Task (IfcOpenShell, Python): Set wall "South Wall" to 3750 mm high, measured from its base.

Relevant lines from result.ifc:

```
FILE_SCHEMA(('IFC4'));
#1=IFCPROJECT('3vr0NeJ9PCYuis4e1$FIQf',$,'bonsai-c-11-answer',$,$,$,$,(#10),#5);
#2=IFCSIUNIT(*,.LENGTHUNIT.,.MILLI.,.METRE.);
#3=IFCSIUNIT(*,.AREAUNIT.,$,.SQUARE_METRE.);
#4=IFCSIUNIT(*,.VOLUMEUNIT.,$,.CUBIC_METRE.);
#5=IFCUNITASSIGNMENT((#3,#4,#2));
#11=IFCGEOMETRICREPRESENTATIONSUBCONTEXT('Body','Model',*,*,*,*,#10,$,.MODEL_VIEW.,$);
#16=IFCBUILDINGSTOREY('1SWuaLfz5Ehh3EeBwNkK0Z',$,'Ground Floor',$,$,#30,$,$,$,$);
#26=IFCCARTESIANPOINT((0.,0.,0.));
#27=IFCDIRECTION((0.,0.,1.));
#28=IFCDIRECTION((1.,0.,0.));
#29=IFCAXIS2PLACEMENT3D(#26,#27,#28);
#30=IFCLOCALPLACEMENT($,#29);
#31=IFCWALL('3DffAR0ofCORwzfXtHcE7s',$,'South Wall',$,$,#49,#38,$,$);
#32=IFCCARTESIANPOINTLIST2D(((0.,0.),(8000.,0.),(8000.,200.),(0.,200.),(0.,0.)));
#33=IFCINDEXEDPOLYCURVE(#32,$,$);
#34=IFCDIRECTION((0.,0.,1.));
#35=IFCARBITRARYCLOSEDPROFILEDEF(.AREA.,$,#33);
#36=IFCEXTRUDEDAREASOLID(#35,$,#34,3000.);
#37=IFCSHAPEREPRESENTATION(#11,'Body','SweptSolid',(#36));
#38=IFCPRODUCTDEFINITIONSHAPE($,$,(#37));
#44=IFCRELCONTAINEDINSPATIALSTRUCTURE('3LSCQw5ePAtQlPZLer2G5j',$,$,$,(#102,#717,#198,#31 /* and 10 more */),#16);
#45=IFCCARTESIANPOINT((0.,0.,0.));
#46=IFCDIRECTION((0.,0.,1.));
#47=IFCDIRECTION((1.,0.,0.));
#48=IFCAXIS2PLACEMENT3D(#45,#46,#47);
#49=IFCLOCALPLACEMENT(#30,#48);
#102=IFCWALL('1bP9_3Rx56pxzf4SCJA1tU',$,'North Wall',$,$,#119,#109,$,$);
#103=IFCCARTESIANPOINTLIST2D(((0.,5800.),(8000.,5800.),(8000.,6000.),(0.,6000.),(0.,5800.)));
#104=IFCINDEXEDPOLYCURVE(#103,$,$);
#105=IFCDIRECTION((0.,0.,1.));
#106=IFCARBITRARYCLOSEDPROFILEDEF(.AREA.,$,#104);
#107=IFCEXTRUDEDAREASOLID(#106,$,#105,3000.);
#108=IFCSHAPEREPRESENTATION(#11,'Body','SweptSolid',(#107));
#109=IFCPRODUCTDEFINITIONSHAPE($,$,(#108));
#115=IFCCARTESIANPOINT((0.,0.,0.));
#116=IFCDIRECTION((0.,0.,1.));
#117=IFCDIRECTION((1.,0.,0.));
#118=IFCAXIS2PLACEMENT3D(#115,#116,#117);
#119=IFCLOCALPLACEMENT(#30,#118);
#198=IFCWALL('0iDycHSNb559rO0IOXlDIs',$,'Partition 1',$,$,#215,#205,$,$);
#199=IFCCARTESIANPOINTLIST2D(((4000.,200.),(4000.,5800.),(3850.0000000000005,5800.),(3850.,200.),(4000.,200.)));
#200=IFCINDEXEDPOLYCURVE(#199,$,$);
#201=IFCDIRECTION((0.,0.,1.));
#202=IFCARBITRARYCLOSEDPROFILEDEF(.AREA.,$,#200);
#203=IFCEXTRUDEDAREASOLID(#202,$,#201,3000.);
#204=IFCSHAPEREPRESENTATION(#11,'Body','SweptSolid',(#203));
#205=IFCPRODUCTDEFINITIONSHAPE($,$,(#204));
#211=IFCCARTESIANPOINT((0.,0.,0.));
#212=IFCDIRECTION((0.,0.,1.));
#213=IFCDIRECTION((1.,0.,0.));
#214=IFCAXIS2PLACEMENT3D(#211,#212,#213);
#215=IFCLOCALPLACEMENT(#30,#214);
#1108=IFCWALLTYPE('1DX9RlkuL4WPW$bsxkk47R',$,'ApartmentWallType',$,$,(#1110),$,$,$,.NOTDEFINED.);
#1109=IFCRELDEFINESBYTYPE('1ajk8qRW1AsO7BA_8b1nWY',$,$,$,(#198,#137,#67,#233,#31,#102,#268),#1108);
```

```python
import ifcopenshell
import ifcopenshell.geom
import ifcopenshell.util.representation
import ifcopenshell.util.shape
import ifcopenshell.util.unit

model = ifcopenshell.open("result.ifc")
unit_scale = ifcopenshell.util.unit.calculate_unit_scale(model)
settings = ifcopenshell.geom.settings()


def volume(element):
    """Net volume in cubic metres, openings subtracted."""
    shape = ifcopenshell.geom.create_shape(settings, element)
    return ifcopenshell.util.shape.get_volume(shape.geometry)


wall = model.by_id(31)
before = volume(wall)

body = ifcopenshell.util.representation.get_representation(wall, "Model", "Body")
solid = body.Items[0]
old_height = solid.Depth
solid.Depth = 3.75 / unit_scale
after = volume(wall)

print(f"height {old_height:g} -> {solid.Depth:g}, volume {before:.3f} -> {after:.3f} m3")

model.write("result_edited.ifc")
```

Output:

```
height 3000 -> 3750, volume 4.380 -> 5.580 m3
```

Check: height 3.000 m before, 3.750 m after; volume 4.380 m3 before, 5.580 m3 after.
